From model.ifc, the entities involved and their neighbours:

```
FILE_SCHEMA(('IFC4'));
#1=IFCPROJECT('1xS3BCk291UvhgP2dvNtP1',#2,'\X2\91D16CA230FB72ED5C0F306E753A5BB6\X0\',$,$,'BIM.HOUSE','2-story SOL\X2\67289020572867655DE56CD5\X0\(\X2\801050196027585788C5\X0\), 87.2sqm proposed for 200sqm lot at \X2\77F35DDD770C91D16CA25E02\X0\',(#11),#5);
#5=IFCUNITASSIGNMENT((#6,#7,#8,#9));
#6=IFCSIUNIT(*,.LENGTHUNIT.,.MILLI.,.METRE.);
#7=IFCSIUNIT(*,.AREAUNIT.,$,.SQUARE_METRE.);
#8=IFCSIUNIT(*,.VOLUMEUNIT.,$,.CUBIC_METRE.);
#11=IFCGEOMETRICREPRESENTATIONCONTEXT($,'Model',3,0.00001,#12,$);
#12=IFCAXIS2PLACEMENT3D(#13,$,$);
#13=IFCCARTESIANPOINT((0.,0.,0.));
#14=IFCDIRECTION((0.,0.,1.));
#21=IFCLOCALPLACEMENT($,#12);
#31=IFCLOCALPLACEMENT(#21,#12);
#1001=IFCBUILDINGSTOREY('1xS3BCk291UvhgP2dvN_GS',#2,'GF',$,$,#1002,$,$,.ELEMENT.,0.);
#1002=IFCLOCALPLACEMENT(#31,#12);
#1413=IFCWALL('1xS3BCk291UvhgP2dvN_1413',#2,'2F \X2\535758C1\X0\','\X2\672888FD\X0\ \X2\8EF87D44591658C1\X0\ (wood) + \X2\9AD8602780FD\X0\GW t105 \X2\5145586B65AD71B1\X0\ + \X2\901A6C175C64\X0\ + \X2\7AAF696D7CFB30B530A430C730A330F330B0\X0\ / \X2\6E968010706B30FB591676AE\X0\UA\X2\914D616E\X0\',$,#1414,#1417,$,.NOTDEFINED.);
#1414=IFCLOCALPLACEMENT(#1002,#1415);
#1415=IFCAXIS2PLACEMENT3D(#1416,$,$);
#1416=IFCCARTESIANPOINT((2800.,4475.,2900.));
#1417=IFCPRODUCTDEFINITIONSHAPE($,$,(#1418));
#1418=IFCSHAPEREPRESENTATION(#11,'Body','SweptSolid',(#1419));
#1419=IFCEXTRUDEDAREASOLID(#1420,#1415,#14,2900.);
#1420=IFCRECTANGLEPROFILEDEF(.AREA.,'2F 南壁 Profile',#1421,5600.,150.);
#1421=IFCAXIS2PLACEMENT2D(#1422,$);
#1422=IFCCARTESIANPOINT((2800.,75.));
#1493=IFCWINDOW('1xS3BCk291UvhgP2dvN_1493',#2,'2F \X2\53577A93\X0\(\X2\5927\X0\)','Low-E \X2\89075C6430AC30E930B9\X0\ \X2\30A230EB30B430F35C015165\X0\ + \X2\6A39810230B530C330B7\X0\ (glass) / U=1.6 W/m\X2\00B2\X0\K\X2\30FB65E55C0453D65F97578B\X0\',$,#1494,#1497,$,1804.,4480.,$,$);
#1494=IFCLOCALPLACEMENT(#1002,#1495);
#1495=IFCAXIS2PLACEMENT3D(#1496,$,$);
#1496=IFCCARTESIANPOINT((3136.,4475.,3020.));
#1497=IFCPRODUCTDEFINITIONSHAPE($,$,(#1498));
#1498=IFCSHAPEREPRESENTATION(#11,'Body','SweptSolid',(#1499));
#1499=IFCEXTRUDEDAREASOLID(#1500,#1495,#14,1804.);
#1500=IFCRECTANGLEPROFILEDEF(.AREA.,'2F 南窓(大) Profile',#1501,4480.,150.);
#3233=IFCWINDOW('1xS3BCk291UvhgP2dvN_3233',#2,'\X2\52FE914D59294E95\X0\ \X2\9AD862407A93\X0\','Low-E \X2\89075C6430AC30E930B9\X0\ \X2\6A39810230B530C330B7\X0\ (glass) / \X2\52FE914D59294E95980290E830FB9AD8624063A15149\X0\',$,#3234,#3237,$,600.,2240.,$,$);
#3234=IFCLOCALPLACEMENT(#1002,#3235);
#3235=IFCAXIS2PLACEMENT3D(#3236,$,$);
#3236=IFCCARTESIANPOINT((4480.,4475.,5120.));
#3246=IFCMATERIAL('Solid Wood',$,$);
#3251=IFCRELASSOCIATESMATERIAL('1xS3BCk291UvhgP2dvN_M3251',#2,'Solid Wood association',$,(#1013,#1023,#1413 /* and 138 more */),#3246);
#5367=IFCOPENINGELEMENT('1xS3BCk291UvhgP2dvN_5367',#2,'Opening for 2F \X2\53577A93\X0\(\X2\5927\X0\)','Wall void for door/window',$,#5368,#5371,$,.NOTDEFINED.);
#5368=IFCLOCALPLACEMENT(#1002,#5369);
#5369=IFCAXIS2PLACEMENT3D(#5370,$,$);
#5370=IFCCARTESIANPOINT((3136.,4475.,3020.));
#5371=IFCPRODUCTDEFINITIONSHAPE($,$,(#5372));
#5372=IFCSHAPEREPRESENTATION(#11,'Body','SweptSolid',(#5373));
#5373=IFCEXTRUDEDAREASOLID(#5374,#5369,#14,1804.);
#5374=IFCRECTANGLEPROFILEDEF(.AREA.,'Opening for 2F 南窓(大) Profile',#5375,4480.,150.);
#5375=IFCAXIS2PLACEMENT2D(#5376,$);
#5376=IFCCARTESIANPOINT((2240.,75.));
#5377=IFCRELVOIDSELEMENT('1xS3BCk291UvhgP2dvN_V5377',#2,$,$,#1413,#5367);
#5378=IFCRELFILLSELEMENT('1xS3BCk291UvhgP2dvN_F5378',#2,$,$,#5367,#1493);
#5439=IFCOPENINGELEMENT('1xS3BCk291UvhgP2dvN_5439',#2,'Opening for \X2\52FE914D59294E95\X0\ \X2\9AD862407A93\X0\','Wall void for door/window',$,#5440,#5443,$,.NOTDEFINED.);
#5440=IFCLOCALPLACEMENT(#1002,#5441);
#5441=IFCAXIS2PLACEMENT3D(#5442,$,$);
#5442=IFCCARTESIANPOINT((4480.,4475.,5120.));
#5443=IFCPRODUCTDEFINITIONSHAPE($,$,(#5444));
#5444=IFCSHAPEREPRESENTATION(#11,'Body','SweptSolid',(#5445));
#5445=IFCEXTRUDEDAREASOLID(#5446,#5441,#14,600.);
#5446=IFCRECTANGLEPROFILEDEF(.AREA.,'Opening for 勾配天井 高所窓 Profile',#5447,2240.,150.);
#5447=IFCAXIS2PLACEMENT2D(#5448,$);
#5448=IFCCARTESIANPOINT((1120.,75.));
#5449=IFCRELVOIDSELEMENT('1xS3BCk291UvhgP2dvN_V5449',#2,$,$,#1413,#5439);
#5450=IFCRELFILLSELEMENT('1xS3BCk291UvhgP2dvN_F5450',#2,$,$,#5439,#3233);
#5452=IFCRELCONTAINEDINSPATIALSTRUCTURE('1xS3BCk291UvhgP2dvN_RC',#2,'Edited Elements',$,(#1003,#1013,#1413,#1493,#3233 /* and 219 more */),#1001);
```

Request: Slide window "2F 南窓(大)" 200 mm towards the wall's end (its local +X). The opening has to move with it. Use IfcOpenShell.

```python
import ifcopenshell
import ifcopenshell.api.geometry
import ifcopenshell.util.placement

model = ifcopenshell.open("model.ifc")

window = model.by_id(1493)
opening = window.FillsVoids[0].RelatingOpeningElement
wall = opening.VoidsElements[0].RelatingBuildingElement

wall_matrix = ifcopenshell.util.placement.get_local_placement(wall.ObjectPlacement)
shift = wall_matrix[:3, 0] * 200.0
before = ifcopenshell.util.placement.get_local_placement(window.ObjectPlacement)[:3, 3].copy()

# The window is not placed relative to its opening, so move both.
for product in (opening, window):
    matrix = ifcopenshell.util.placement.get_local_placement(product.ObjectPlacement)
    matrix[:3, 3] += shift
    ifcopenshell.api.geometry.edit_object_placement(model, product=product, matrix=matrix, is_si=False)

after = ifcopenshell.util.placement.get_local_placement(window.ObjectPlacement)[:3, 3]
print("window moved by", (after - before).round(3) + 0.0)

model.write("model_rev.ifc")
```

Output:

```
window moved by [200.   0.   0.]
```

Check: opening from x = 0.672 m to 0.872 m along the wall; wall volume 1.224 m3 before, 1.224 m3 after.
